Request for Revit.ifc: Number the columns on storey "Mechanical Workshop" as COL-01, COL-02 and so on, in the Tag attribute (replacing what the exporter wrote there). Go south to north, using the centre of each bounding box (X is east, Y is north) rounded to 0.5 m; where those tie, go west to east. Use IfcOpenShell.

First a look at what the model holds.

```python
import ifcopenshell
import ifcopenshell.util.element
import ifcopenshell.util.placement

model = ifcopenshell.open("Revit.ifc")
print(model.schema)
storey = next(s for s in model.by_type("IfcBuildingStorey") if s.Name == "Mechanical Workshop")
columns = [e for e in ifcopenshell.util.element.get_decomposition(storey) if e.is_a("IfcColumn")]
for e in sorted(columns, key=lambda e: e.id()):
    origin = ifcopenshell.util.placement.get_local_placement(e.ObjectPlacement)[:3, 3]
    print(e.id(), e.Tag, e.Name, origin.round(2) + 0.0, sep=" | ")
```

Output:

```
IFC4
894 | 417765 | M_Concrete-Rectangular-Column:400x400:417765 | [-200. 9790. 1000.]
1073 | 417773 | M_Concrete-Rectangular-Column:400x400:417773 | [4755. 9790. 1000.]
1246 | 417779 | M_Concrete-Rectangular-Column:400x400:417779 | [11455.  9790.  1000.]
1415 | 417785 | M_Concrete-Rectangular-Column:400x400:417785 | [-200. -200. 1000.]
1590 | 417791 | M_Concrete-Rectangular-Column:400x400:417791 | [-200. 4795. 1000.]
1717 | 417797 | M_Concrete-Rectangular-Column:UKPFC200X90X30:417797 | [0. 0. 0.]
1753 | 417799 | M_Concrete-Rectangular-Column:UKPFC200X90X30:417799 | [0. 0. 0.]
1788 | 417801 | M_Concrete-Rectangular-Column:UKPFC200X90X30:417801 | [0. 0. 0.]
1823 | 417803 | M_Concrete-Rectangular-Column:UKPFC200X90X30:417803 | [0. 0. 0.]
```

```python
import ifcopenshell
import ifcopenshell.geom
import ifcopenshell.util.element
import ifcopenshell.util.shape

model = ifcopenshell.open("Revit.ifc")
settings = ifcopenshell.geom.settings()
settings.set("use-world-coords", True)


def centre(element):
    shape = ifcopenshell.geom.create_shape(settings, element)
    return ifcopenshell.util.shape.get_bbox_centroid(shape.geometry)


storey = next(s for s in model.by_type("IfcBuildingStorey") if s.Name == "Mechanical Workshop")
columns = [e for e in ifcopenshell.util.element.get_decomposition(storey) if e.is_a("IfcColumn")]

# Insertion points can sit at a corner or the storey origin, so sort by the geometry (in metres).
centres = {e: centre(e) for e in columns}
columns.sort(key=lambda e: (round(centres[e][1] / 0.5), centres[e][0]))

for i, e in enumerate(columns, start=1):
    number = f"COL-{i:02d}"
    e.Tag = number
    print(e.id(), number)

model.write("Revit_v2.ifc")
```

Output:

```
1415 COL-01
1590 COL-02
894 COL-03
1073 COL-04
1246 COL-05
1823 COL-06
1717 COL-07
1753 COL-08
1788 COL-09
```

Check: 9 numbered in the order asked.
